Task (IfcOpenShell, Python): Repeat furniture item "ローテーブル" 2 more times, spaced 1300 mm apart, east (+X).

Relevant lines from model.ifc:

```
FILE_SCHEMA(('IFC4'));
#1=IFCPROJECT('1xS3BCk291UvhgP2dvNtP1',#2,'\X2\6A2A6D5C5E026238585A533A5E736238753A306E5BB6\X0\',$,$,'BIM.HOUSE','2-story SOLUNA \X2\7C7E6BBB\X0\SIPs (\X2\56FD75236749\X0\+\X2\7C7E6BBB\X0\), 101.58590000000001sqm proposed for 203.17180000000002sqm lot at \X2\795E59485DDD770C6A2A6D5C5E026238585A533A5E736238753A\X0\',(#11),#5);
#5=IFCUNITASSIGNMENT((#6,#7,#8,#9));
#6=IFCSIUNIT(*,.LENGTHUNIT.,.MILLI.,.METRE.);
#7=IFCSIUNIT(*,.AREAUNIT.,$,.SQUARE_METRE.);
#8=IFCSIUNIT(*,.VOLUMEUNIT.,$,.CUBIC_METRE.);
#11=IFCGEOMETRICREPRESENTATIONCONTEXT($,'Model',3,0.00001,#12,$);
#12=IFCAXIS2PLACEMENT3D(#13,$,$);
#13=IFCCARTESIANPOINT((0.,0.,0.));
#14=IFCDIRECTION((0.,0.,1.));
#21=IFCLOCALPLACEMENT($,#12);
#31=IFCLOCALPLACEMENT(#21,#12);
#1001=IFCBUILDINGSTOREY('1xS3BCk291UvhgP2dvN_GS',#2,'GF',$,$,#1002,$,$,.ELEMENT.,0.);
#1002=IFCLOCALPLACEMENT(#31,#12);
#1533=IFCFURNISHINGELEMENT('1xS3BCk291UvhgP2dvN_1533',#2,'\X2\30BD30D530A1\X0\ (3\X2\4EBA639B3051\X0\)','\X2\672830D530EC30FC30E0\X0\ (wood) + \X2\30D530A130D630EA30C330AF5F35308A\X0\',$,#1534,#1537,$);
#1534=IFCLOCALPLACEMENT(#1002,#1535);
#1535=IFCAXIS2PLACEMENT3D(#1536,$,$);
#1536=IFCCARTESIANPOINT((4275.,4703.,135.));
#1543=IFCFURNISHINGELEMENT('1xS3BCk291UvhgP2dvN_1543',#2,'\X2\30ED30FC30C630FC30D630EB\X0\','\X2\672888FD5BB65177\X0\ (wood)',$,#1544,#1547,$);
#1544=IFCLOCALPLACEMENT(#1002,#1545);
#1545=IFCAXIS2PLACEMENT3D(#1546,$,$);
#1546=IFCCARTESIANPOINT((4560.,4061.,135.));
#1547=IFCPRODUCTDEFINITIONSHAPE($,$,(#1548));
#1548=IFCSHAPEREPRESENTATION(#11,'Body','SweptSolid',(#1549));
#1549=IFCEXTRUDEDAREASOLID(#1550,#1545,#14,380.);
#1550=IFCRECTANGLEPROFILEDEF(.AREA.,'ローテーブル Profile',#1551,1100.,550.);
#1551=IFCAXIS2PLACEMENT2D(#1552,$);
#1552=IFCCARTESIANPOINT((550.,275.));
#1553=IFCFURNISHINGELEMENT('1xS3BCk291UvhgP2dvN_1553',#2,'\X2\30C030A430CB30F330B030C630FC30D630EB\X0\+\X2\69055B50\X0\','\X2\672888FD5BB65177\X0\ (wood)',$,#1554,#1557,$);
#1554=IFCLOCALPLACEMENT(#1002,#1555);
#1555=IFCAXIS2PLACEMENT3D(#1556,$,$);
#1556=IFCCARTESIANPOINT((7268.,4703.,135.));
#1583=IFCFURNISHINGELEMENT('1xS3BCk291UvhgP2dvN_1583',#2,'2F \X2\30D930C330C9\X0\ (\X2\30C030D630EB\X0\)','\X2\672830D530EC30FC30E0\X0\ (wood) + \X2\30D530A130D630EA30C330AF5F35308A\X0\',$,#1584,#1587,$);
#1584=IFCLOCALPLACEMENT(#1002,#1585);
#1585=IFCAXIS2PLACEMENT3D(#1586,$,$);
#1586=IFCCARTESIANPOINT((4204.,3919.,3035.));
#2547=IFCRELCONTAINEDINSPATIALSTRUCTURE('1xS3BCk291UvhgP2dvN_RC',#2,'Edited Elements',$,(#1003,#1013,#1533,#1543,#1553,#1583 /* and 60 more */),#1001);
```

```python
import numpy as np
import ifcopenshell
import ifcopenshell.api.geometry
import ifcopenshell.api.root
import ifcopenshell.util.element
import ifcopenshell.util.placement
import ifcopenshell.util.unit

model = ifcopenshell.open("model.ifc")
unit_scale = ifcopenshell.util.unit.calculate_unit_scale(model)


def reuse_history(source, copy):
    """copy_class also copies each property set's owner history, people and application; keep the originals."""
    for rel in copy.IsDefinedBy:
        if rel.is_a("IfcRelDefinesByProperties") and (history := rel.RelatingPropertyDefinition.OwnerHistory):
            rel.RelatingPropertyDefinition.OwnerHistory = source.OwnerHistory
            ifcopenshell.util.element.remove_deep2(model, history)


source = model.by_guid("1xS3BCk291UvhgP2dvN_1543")
base = ifcopenshell.util.placement.get_local_placement(source.ObjectPlacement)
step = np.array([1.0, 0.0, 0.0]) * 1.3 / unit_scale

for i in range(1, 3):
    copy = ifcopenshell.api.root.copy_class(model, product=source)
    copy.Representation = ifcopenshell.util.element.copy_deep(
        model, source.Representation, exclude=["IfcGeometricRepresentationContext", "IfcRepresentationMap"]
    )
    reuse_history(source, copy)
    matrix = base.copy()
    matrix[:3, 3] += i * step
    print("added at", matrix[:3, 3].round(3) + 0.0)
    ifcopenshell.api.geometry.edit_object_placement(model, product=copy, matrix=matrix, is_si=False)

model.write("model-out.ifc")
```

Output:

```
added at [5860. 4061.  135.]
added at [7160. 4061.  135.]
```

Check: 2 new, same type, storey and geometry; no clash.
